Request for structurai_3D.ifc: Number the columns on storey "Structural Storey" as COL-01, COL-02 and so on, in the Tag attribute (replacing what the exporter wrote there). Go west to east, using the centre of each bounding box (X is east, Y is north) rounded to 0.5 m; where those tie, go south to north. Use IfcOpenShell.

First a look at what the model holds.

```python
import ifcopenshell
import ifcopenshell.util.element
import ifcopenshell.util.placement

model = ifcopenshell.open("structurai_3D.ifc")
print(model.schema)
storey = next(s for s in model.by_type("IfcBuildingStorey") if s.Name == "Structural Storey")
columns = [e for e in ifcopenshell.util.element.get_decomposition(storey) if e.is_a("IfcColumn")]
for e in sorted(columns, key=lambda e: e.id()):
    origin = ifcopenshell.util.placement.get_local_placement(e.ObjectPlacement)[:3, 3]
    print(e.id(), e.Tag, e.Name, origin.round(2) + 0.0, sep=" | ")
```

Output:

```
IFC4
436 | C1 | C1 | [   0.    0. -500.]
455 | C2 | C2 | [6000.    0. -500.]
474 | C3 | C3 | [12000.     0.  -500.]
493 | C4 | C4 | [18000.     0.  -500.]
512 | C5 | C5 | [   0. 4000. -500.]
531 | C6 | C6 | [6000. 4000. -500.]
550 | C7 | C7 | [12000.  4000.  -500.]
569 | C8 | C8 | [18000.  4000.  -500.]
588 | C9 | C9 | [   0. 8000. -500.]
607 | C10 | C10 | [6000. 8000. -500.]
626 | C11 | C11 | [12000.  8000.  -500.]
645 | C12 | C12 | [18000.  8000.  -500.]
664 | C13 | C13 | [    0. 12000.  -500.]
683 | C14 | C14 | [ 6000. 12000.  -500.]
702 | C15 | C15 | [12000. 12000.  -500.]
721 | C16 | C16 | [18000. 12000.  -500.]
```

```python
import ifcopenshell
import ifcopenshell.geom
import ifcopenshell.util.element
import ifcopenshell.util.shape

model = ifcopenshell.open("structurai_3D.ifc")
settings = ifcopenshell.geom.settings()
settings.set("use-world-coords", True)


def centre(element):
    shape = ifcopenshell.geom.create_shape(settings, element)
    return ifcopenshell.util.shape.get_bbox_centroid(shape.geometry)


storey = next(s for s in model.by_type("IfcBuildingStorey") if s.Name == "Structural Storey")
columns = [e for e in ifcopenshell.util.element.get_decomposition(storey) if e.is_a("IfcColumn")]

# Insertion points can sit at a corner or the storey origin, so sort by the geometry (in metres).
centres = {e: centre(e) for e in columns}
columns.sort(key=lambda e: (round(centres[e][0] / 0.5), centres[e][1]))

for i, e in enumerate(columns, start=1):
    number = f"COL-{i:02d}"
    e.Tag = number
    print(e.id(), number)

model.write("structurai_3D_v2.ifc")
```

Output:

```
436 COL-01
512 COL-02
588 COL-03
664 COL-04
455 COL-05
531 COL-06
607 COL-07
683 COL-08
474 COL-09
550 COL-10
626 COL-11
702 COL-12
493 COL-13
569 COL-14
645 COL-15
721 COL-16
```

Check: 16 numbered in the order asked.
